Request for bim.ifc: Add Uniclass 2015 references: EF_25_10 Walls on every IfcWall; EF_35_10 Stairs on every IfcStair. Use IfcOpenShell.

First a look at what the model holds.

```python
import ifcopenshell

model = ifcopenshell.open("bim.ifc")
print(model.schema)
print("classifications:", [c.Name for c in model.by_type("IfcClassification")])
for ifc_class in ("IfcDoor", "IfcRoof", "IfcStair", "IfcWall", "IfcWindow"):
    print(ifc_class, len(model.by_type(ifc_class)))
```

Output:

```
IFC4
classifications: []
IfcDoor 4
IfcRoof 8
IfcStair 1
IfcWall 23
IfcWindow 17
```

```python
import ifcopenshell
import ifcopenshell.api.classification

model = ifcopenshell.open("bim.ifc")

system = ifcopenshell.api.classification.add_classification(model, classification="Uniclass 2015")

codes = {
    "IfcWall": ("EF_25_10", "Walls"),
    "IfcStair": ("EF_35_10", "Stairs"),
}
for ifc_class, (code, name) in codes.items():
    products = model.by_type(ifc_class)
    ifcopenshell.api.classification.add_reference(
        model, products=products, classification=system, identification=code, name=name
    )
    print(code, len(products))

model.write("bim_rev.ifc")
```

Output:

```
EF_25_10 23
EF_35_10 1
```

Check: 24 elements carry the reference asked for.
